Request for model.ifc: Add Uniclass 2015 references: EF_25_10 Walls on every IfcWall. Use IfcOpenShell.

First a look at what the model holds.

```python
import ifcopenshell

model = ifcopenshell.open("model.ifc")
print(model.schema)
print("classifications:", [c.Name for c in model.by_type("IfcClassification")])
for ifc_class in ("IfcDoor", "IfcRoof", "IfcStair", "IfcWall", "IfcWindow"):
    print(ifc_class, len(model.by_type(ifc_class)))
```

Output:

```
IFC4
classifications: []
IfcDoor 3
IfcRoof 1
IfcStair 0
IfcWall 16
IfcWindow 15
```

```python
import ifcopenshell
import ifcopenshell.api.classification

model = ifcopenshell.open("model.ifc")

system = ifcopenshell.api.classification.add_classification(model, classification="Uniclass 2015")

codes = {
    "IfcWall": ("EF_25_10", "Walls"),
}
for ifc_class, (code, name) in codes.items():
    products = model.by_type(ifc_class)
    ifcopenshell.api.classification.add_reference(
        model, products=products, classification=system, identification=code, name=name
    )
    print(code, len(products))

model.write("model-out.ifc")
```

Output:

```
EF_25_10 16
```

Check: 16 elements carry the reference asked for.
